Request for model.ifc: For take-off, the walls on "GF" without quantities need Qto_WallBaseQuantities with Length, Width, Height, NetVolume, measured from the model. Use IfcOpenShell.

First a look at what the model holds.

```python
import ifcopenshell
import ifcopenshell.util.element
import ifcopenshell.util.unit

model = ifcopenshell.open("model.ifc")
print(model.schema)
for unit_type in ("LENGTHUNIT", "AREAUNIT", "VOLUMEUNIT"):
    print(unit_type, ifcopenshell.util.unit.calculate_unit_scale(model, unit_type))
storey = next(s for s in model.by_type("IfcBuildingStorey") if s.Name == "GF")
walls = [e for e in ifcopenshell.util.element.get_decomposition(storey) if e.is_a("IfcWall")]
for e in sorted(walls, key=lambda e: e.id()):
    print(e.id(), e.is_a(), e.Name, list(ifcopenshell.util.element.get_psets(e, qtos_only=True)), sep=" | ")
```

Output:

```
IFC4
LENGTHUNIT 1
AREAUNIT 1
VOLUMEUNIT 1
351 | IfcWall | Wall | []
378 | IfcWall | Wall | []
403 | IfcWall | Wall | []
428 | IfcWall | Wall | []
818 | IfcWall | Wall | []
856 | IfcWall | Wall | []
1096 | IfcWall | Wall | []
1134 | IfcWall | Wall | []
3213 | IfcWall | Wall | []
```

```python
import ifcopenshell
import ifcopenshell.api.pset
import ifcopenshell.geom
import ifcopenshell.util.element
import ifcopenshell.util.shape
import ifcopenshell.util.unit

model = ifcopenshell.open("model.ifc")
unit_scale = ifcopenshell.util.unit.calculate_unit_scale(model)
volume_scale = ifcopenshell.util.unit.calculate_unit_scale(model, "VOLUMEUNIT")
settings = ifcopenshell.geom.settings()

storey = next(s for s in model.by_type("IfcBuildingStorey") if s.Name == "GF")
walls = [e for e in ifcopenshell.util.element.get_decomposition(storey) if e.is_a("IfcWall")]

for e in sorted(walls, key=lambda e: e.id()):
    if ifcopenshell.util.element.get_psets(e, qtos_only=True, should_inherit=False):
        continue
    # Geometry comes back in metres, in the element's own axes.
    shape = ifcopenshell.geom.create_shape(settings, e)
    values = {
        "Length": ifcopenshell.util.shape.get_x(shape.geometry) / unit_scale,
        "Width": ifcopenshell.util.shape.get_y(shape.geometry) / unit_scale,
        "Height": ifcopenshell.util.shape.get_z(shape.geometry) / unit_scale,
        "NetVolume": ifcopenshell.util.shape.get_volume(shape.geometry) / volume_scale,
    }
    qto = ifcopenshell.api.pset.add_qto(model, product=e, name="Qto_WallBaseQuantities")
    ifcopenshell.api.pset.edit_qto(model, qto=qto, properties=values)
    print(e.id(), {k: round(v, 3) for k, v in values.items()})

model.write("model_updated.ifc")
```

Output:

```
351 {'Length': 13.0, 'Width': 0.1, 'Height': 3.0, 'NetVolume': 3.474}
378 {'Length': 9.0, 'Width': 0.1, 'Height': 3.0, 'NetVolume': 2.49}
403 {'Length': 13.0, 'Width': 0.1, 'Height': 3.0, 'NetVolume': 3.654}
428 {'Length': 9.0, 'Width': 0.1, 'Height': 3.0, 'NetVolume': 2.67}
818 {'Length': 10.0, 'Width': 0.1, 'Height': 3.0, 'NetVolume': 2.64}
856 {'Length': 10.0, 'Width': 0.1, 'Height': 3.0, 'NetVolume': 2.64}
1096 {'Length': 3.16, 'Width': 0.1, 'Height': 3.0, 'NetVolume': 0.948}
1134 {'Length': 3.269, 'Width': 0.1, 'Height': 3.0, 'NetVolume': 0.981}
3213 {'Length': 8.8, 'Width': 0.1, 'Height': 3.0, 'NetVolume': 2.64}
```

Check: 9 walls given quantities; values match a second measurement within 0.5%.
